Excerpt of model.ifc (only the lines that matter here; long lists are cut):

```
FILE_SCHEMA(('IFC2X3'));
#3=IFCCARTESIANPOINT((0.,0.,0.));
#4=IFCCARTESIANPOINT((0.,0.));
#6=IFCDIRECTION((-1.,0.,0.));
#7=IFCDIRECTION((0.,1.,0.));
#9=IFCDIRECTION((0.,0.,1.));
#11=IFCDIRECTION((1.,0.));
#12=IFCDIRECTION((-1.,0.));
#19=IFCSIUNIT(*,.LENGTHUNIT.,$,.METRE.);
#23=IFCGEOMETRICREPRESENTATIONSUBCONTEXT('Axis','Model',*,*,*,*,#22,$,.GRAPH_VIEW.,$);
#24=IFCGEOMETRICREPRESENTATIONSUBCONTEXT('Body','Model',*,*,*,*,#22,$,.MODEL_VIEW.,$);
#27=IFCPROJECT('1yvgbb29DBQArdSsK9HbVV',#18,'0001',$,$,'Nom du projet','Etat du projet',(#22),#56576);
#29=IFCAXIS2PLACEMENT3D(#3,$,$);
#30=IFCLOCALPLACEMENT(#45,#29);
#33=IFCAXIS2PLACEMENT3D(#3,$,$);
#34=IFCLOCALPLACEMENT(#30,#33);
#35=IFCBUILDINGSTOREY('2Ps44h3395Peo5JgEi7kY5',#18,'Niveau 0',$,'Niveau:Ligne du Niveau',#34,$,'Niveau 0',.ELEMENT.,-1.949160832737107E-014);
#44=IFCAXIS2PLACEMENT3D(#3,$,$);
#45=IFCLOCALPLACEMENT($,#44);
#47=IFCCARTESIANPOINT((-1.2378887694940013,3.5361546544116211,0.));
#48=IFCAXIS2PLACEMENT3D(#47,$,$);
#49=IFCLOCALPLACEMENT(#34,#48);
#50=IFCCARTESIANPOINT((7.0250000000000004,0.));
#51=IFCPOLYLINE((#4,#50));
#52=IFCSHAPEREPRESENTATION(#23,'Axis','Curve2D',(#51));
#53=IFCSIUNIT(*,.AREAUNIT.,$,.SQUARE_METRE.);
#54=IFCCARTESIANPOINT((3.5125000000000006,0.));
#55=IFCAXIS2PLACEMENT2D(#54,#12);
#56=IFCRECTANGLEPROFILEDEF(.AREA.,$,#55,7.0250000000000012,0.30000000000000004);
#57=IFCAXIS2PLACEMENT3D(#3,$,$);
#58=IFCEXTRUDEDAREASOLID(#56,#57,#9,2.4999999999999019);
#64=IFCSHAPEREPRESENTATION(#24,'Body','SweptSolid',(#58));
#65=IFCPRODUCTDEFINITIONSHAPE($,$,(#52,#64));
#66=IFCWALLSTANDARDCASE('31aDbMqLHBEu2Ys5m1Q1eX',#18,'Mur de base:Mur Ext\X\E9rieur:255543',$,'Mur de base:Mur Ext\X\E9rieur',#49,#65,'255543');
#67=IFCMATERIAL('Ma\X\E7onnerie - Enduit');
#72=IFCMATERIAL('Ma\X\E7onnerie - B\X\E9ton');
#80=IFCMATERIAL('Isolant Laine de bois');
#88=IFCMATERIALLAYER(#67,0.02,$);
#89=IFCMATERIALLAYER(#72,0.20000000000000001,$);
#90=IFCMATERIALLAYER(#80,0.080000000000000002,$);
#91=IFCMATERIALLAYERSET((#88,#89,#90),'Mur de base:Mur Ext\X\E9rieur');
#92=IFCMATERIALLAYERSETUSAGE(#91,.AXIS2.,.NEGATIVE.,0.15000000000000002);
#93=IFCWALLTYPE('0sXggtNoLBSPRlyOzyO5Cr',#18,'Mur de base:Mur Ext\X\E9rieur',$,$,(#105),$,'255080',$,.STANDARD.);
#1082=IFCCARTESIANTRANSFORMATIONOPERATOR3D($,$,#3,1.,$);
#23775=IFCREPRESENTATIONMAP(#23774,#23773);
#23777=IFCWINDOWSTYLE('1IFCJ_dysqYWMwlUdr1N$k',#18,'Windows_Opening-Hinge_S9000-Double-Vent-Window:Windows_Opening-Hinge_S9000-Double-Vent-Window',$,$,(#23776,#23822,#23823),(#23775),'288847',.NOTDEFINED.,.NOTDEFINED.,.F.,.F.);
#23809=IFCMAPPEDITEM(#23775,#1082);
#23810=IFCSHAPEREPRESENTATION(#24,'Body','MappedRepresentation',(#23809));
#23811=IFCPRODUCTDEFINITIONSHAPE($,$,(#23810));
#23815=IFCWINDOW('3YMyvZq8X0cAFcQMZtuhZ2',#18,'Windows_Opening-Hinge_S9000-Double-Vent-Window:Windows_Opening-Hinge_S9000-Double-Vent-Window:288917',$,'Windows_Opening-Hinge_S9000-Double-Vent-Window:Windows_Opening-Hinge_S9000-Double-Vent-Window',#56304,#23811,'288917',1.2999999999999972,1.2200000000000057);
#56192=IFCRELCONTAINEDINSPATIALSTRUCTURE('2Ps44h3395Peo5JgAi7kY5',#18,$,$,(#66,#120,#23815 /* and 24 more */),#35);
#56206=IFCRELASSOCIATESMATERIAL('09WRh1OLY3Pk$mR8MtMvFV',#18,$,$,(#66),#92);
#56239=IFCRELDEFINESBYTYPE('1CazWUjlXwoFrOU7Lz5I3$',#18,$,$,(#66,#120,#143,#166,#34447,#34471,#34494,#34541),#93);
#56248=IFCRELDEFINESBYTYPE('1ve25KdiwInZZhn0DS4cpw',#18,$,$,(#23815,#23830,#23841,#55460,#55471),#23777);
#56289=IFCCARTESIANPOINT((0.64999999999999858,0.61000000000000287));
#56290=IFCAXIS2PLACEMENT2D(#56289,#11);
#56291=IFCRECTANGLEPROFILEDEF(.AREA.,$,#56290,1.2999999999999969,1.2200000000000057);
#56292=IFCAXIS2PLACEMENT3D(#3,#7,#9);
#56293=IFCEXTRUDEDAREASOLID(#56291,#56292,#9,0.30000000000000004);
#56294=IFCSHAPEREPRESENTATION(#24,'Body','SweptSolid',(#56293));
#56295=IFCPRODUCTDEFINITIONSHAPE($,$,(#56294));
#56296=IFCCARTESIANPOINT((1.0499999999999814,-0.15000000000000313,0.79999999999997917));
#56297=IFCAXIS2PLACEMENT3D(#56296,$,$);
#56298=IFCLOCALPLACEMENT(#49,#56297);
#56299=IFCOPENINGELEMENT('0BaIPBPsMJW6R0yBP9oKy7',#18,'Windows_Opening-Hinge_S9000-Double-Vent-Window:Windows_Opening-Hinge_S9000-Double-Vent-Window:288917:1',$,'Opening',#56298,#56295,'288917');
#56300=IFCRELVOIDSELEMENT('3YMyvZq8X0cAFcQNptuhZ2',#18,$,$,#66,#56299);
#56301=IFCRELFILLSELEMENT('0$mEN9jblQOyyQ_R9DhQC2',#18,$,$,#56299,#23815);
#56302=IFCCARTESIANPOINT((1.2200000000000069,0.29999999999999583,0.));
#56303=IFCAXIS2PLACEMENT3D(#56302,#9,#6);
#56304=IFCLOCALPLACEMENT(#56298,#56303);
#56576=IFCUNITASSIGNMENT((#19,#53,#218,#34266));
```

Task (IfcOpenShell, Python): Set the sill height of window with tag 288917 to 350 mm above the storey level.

```python
import numpy as np
import ifcopenshell
import ifcopenshell.api.geometry
import ifcopenshell.geom
import ifcopenshell.util.element
import ifcopenshell.util.placement
import ifcopenshell.util.shape
import ifcopenshell.util.unit

model = ifcopenshell.open("model.ifc")
unit_scale = ifcopenshell.util.unit.calculate_unit_scale(model)

window = model.by_guid("3YMyvZq8X0cAFcQMZtuhZ2")
opening = window.FillsVoids[0].RelatingOpeningElement
storey = ifcopenshell.util.element.get_container(window, ifc_class="IfcBuildingStorey")
level = ifcopenshell.util.placement.get_local_placement(storey.ObjectPlacement)[2, 3]

# The opening's origin need not be at the sill, so measure its lowest point.
shape = ifcopenshell.geom.create_shape(ifcopenshell.geom.settings(), opening)
bottom = ifcopenshell.util.shape.get_shape_bottom_elevation(shape, shape.geometry) / unit_scale
dz = level + 0.35 - bottom

shift = np.array([0.0, 0.0, dz])
# The window is placed relative to its opening, so it follows when the opening moves.
matrix = ifcopenshell.util.placement.get_local_placement(opening.ObjectPlacement)
matrix[:3, 3] += shift
ifcopenshell.api.geometry.edit_object_placement(
    model, product=opening, matrix=matrix, is_si=False, should_transform_children=True
)

print(f"moved by {dz * unit_scale:+.3f} m")

model.write("model_edited.ifc")
```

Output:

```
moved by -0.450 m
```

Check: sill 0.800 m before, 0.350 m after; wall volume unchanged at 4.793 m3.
